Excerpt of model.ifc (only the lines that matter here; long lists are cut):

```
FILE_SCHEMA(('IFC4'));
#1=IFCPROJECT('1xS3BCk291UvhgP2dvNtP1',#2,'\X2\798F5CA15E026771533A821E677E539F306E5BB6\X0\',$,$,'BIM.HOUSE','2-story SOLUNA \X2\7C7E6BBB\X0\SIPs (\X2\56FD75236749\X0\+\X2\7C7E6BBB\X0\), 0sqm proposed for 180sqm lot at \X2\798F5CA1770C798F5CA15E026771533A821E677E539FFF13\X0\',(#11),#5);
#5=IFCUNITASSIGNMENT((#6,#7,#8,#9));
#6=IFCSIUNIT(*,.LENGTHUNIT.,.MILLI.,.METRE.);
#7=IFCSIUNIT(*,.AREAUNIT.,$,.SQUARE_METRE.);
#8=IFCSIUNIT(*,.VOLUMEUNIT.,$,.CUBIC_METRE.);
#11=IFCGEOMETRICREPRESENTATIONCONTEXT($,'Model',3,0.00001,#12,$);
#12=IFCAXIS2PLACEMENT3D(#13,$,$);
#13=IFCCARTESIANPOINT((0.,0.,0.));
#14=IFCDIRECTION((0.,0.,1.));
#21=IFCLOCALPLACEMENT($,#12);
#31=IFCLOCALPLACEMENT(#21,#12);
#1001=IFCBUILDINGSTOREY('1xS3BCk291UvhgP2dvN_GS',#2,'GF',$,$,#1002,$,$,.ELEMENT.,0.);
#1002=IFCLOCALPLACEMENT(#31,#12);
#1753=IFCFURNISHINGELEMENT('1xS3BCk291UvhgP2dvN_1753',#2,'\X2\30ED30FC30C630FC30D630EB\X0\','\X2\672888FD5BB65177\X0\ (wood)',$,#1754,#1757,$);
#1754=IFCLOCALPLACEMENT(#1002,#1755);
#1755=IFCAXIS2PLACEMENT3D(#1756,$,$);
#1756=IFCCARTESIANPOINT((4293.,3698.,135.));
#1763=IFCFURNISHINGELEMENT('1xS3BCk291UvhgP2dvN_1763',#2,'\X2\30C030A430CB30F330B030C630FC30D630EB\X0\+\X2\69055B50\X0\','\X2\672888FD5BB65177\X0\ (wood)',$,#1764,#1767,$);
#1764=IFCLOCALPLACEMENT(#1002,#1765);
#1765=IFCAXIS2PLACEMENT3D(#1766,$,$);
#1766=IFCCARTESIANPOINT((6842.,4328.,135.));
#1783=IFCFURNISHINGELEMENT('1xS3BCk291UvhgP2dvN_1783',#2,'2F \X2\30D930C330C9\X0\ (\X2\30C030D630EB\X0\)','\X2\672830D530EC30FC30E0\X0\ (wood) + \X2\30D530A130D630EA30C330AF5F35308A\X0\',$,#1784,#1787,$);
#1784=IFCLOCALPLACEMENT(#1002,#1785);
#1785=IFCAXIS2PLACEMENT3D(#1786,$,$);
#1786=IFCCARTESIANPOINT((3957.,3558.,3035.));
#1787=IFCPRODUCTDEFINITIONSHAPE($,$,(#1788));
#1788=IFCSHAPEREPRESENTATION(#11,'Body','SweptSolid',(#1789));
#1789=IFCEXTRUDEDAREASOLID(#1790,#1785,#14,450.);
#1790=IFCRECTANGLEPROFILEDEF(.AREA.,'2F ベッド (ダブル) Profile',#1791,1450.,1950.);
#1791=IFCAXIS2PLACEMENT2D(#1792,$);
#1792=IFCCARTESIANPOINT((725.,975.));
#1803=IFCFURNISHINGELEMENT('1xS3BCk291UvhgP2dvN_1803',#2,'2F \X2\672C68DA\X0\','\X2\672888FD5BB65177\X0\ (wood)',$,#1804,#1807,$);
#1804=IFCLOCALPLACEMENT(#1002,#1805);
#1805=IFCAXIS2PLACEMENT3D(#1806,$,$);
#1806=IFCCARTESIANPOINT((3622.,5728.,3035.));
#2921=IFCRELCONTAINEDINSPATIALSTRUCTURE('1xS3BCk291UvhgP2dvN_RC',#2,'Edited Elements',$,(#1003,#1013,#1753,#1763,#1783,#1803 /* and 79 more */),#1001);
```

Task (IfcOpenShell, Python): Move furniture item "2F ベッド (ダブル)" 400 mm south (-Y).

```python
import ifcopenshell
import ifcopenshell.api.geometry
import ifcopenshell.util.placement
import ifcopenshell.util.unit

model = ifcopenshell.open("model.ifc")
unit_scale = ifcopenshell.util.unit.calculate_unit_scale(model)

item = model.by_guid("1xS3BCk291UvhgP2dvN_1783")
matrix = ifcopenshell.util.placement.get_local_placement(item.ObjectPlacement)
matrix[1, 3] -= 0.4 / unit_scale
ifcopenshell.api.geometry.edit_object_placement(model, product=item, matrix=matrix, is_si=False)

print(ifcopenshell.util.placement.get_local_placement(item.ObjectPlacement).round(3) + 0.0)

model.write("model_rev.ifc")
```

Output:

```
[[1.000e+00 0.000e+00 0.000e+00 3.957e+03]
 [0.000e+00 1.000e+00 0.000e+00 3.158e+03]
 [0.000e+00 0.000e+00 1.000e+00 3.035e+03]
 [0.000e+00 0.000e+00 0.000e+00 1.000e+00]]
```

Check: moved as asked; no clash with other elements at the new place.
